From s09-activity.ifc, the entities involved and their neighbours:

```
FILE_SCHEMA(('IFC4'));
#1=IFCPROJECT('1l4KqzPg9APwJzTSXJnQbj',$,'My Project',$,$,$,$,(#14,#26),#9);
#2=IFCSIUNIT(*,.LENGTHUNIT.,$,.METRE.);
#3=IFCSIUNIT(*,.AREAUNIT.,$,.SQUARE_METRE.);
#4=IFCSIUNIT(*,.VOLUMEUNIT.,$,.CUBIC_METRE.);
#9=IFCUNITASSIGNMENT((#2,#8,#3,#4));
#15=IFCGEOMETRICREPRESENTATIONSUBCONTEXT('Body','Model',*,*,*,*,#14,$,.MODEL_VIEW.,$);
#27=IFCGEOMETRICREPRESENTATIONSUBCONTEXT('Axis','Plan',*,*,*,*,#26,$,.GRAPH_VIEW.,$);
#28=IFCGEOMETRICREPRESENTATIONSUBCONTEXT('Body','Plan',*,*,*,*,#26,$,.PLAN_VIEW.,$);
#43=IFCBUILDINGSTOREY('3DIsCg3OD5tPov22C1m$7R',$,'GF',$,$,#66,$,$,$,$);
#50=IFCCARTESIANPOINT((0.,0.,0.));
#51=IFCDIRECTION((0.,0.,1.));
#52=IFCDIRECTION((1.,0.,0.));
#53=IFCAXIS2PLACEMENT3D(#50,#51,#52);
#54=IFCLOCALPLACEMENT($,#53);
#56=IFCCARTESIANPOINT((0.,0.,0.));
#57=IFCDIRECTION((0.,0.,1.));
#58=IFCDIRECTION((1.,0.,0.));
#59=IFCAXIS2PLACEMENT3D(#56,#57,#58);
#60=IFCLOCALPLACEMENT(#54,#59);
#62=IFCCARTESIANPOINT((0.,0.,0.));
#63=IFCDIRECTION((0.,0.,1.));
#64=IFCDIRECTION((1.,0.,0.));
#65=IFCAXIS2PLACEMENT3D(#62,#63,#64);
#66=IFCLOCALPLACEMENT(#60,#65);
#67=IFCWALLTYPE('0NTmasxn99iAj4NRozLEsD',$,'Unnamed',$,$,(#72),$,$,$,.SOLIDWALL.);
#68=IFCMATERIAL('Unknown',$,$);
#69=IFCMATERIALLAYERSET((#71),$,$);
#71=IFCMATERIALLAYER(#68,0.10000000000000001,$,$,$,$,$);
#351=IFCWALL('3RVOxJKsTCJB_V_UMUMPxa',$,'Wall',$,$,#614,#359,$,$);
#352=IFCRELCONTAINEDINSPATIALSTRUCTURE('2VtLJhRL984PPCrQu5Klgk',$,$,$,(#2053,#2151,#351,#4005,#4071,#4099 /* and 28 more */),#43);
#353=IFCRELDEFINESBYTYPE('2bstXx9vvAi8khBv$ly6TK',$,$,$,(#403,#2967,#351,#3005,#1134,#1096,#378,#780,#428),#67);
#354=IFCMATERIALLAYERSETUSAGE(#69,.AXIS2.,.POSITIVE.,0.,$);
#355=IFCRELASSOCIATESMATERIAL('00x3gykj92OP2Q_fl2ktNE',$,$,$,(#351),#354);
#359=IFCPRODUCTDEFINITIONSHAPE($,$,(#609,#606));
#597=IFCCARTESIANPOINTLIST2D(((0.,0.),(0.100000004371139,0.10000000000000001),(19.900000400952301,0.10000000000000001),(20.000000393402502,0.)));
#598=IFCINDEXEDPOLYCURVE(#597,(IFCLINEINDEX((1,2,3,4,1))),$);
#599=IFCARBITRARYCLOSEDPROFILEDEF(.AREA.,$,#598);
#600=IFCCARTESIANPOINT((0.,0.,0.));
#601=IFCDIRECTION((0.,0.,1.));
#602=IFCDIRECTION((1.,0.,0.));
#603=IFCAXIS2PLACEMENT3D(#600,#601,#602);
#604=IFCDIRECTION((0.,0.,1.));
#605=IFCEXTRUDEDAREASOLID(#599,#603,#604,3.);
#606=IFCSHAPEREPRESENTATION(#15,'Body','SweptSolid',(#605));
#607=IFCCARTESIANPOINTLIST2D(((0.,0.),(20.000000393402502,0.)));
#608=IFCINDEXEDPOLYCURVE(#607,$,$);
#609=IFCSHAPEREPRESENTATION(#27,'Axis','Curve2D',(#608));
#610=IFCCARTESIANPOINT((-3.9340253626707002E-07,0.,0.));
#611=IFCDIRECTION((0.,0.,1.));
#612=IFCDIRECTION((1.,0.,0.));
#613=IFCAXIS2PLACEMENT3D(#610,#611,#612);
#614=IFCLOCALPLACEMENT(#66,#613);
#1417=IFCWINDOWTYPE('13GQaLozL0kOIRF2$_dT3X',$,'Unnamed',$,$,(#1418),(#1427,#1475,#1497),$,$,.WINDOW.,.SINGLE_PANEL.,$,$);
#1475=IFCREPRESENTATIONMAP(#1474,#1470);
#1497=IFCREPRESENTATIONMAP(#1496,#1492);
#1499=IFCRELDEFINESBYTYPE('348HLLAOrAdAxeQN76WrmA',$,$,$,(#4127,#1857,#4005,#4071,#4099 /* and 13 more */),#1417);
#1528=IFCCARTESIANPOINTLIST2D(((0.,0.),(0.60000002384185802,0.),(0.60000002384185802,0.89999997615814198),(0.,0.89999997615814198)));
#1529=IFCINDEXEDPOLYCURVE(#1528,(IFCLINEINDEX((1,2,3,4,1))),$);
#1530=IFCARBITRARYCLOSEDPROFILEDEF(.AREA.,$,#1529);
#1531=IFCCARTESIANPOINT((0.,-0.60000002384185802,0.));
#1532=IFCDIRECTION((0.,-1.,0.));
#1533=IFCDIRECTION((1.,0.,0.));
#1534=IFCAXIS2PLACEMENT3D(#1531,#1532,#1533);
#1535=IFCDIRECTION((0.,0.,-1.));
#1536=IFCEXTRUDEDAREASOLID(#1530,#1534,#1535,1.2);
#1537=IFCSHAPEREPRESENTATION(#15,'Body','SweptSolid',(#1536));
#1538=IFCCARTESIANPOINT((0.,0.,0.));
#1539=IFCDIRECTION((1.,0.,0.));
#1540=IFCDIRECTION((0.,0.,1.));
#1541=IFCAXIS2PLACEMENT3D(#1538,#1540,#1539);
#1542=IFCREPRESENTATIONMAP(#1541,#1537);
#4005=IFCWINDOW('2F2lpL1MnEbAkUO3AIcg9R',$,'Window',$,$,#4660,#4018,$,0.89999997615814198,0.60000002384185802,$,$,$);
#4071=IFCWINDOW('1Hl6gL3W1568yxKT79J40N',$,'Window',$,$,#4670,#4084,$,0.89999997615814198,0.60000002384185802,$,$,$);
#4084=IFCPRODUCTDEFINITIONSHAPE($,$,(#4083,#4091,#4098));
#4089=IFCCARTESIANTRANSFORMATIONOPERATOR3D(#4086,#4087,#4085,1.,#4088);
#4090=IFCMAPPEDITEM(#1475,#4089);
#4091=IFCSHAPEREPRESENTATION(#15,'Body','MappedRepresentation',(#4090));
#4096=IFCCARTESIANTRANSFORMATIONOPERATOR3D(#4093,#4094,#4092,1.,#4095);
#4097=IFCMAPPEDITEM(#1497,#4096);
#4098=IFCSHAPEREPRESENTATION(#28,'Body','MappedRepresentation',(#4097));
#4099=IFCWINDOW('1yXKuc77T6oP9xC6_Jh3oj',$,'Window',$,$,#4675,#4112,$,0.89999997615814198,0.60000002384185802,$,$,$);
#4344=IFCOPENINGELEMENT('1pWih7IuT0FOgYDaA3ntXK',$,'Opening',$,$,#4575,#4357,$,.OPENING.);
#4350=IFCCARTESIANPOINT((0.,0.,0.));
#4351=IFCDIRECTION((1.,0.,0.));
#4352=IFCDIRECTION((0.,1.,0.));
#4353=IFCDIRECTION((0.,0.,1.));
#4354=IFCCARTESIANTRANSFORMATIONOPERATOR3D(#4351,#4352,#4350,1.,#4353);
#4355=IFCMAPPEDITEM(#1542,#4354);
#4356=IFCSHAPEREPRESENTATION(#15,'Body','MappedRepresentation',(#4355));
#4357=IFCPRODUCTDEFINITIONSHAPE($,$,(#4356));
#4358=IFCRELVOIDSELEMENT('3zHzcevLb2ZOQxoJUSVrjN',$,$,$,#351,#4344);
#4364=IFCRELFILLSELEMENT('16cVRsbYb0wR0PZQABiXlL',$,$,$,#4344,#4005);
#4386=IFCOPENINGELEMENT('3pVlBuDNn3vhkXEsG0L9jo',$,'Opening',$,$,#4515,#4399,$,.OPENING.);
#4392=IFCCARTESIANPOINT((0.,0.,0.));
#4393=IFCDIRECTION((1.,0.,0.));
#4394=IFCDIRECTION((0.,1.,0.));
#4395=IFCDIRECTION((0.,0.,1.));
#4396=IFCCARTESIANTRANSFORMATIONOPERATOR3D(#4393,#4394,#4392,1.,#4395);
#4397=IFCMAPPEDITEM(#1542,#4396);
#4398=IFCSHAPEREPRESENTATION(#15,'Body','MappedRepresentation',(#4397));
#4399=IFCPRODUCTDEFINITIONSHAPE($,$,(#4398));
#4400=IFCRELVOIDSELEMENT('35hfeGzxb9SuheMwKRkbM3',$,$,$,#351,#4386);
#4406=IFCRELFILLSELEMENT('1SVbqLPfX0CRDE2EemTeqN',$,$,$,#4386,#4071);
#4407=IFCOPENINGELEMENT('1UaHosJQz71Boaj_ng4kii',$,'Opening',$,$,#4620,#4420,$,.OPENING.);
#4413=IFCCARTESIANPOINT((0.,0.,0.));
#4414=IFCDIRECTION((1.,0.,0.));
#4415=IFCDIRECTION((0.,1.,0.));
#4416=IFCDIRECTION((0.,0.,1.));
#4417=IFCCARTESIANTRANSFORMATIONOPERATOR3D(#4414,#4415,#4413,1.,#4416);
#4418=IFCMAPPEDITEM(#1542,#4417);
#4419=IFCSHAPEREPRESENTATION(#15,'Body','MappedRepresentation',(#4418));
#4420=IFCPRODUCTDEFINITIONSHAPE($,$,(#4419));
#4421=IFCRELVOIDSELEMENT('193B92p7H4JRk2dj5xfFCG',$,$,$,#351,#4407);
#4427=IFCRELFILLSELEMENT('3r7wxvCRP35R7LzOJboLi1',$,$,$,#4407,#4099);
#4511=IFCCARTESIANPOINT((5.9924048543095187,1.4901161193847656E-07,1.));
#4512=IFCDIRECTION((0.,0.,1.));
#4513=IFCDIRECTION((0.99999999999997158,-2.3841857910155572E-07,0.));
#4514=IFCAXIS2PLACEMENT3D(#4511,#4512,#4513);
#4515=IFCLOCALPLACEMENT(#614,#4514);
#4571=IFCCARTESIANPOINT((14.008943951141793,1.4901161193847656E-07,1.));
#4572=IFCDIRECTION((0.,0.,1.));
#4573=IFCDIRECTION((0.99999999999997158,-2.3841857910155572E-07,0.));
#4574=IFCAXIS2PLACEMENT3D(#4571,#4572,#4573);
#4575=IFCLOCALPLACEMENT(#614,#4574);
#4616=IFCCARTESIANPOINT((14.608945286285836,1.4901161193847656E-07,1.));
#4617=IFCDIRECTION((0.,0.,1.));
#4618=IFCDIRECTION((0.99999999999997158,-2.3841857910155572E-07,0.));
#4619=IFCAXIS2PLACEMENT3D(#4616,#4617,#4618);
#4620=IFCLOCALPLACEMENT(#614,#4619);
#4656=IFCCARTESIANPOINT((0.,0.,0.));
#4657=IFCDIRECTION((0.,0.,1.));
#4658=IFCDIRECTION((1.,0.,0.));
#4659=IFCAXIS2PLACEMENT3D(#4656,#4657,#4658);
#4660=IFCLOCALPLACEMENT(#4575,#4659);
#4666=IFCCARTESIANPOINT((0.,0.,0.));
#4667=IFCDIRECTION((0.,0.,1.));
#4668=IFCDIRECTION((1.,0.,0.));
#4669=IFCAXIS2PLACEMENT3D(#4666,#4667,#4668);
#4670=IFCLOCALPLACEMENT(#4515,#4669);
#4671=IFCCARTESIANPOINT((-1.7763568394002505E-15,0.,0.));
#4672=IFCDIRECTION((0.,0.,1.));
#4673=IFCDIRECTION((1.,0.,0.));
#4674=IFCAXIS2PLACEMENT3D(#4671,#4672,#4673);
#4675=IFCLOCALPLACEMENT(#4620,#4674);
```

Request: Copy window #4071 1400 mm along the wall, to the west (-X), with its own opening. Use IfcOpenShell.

```python
import ifcopenshell
import ifcopenshell.api.feature
import ifcopenshell.api.geometry
import ifcopenshell.api.root
import ifcopenshell.geom
import ifcopenshell.util.element
import ifcopenshell.util.placement
import ifcopenshell.util.shape
import ifcopenshell.util.unit

model = ifcopenshell.open("s09-activity.ifc")
unit_scale = ifcopenshell.util.unit.calculate_unit_scale(model)
settings = ifcopenshell.geom.settings()


def volume(element):
    """Net volume in cubic metres, openings subtracted."""
    shape = ifcopenshell.geom.create_shape(settings, element)
    return ifcopenshell.util.shape.get_volume(shape.geometry)


window = model.by_guid("1Hl6gL3W1568yxKT79J40N")
opening = window.FillsVoids[0].RelatingOpeningElement
wall = opening.VoidsElements[0].RelatingBuildingElement
before = volume(wall)
shift = ifcopenshell.util.placement.get_local_placement(wall.ObjectPlacement)[:3, 0] * -1.4 / unit_scale

# copy_class copies the void relationship, type, container and properties, but no geometry.
new_opening = ifcopenshell.api.root.copy_class(model, product=opening)
new_opening.Representation = ifcopenshell.util.element.copy_deep(
    model, opening.Representation, exclude=["IfcGeometricRepresentationContext", "IfcRepresentationMap"]
)
new_window = ifcopenshell.api.root.copy_class(model, product=window)
new_window.Representation = ifcopenshell.util.element.copy_deep(
    model, window.Representation, exclude=["IfcGeometricRepresentationContext", "IfcRepresentationMap"]
)
ifcopenshell.api.feature.add_filling(model, opening=new_opening, element=new_window)

for old, new in ((opening, new_opening), (window, new_window)):
    matrix = ifcopenshell.util.placement.get_local_placement(old.ObjectPlacement)
    matrix[:3, 3] += shift
    ifcopenshell.api.geometry.edit_object_placement(model, product=new, matrix=matrix, is_si=False)

after = volume(wall)

print(f"wall volume {before:.3f} -> {after:.3f} m3")

model.write("s09-activity_rev.ifc")
```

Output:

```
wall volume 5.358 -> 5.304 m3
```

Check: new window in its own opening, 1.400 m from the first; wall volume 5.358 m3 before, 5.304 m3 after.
